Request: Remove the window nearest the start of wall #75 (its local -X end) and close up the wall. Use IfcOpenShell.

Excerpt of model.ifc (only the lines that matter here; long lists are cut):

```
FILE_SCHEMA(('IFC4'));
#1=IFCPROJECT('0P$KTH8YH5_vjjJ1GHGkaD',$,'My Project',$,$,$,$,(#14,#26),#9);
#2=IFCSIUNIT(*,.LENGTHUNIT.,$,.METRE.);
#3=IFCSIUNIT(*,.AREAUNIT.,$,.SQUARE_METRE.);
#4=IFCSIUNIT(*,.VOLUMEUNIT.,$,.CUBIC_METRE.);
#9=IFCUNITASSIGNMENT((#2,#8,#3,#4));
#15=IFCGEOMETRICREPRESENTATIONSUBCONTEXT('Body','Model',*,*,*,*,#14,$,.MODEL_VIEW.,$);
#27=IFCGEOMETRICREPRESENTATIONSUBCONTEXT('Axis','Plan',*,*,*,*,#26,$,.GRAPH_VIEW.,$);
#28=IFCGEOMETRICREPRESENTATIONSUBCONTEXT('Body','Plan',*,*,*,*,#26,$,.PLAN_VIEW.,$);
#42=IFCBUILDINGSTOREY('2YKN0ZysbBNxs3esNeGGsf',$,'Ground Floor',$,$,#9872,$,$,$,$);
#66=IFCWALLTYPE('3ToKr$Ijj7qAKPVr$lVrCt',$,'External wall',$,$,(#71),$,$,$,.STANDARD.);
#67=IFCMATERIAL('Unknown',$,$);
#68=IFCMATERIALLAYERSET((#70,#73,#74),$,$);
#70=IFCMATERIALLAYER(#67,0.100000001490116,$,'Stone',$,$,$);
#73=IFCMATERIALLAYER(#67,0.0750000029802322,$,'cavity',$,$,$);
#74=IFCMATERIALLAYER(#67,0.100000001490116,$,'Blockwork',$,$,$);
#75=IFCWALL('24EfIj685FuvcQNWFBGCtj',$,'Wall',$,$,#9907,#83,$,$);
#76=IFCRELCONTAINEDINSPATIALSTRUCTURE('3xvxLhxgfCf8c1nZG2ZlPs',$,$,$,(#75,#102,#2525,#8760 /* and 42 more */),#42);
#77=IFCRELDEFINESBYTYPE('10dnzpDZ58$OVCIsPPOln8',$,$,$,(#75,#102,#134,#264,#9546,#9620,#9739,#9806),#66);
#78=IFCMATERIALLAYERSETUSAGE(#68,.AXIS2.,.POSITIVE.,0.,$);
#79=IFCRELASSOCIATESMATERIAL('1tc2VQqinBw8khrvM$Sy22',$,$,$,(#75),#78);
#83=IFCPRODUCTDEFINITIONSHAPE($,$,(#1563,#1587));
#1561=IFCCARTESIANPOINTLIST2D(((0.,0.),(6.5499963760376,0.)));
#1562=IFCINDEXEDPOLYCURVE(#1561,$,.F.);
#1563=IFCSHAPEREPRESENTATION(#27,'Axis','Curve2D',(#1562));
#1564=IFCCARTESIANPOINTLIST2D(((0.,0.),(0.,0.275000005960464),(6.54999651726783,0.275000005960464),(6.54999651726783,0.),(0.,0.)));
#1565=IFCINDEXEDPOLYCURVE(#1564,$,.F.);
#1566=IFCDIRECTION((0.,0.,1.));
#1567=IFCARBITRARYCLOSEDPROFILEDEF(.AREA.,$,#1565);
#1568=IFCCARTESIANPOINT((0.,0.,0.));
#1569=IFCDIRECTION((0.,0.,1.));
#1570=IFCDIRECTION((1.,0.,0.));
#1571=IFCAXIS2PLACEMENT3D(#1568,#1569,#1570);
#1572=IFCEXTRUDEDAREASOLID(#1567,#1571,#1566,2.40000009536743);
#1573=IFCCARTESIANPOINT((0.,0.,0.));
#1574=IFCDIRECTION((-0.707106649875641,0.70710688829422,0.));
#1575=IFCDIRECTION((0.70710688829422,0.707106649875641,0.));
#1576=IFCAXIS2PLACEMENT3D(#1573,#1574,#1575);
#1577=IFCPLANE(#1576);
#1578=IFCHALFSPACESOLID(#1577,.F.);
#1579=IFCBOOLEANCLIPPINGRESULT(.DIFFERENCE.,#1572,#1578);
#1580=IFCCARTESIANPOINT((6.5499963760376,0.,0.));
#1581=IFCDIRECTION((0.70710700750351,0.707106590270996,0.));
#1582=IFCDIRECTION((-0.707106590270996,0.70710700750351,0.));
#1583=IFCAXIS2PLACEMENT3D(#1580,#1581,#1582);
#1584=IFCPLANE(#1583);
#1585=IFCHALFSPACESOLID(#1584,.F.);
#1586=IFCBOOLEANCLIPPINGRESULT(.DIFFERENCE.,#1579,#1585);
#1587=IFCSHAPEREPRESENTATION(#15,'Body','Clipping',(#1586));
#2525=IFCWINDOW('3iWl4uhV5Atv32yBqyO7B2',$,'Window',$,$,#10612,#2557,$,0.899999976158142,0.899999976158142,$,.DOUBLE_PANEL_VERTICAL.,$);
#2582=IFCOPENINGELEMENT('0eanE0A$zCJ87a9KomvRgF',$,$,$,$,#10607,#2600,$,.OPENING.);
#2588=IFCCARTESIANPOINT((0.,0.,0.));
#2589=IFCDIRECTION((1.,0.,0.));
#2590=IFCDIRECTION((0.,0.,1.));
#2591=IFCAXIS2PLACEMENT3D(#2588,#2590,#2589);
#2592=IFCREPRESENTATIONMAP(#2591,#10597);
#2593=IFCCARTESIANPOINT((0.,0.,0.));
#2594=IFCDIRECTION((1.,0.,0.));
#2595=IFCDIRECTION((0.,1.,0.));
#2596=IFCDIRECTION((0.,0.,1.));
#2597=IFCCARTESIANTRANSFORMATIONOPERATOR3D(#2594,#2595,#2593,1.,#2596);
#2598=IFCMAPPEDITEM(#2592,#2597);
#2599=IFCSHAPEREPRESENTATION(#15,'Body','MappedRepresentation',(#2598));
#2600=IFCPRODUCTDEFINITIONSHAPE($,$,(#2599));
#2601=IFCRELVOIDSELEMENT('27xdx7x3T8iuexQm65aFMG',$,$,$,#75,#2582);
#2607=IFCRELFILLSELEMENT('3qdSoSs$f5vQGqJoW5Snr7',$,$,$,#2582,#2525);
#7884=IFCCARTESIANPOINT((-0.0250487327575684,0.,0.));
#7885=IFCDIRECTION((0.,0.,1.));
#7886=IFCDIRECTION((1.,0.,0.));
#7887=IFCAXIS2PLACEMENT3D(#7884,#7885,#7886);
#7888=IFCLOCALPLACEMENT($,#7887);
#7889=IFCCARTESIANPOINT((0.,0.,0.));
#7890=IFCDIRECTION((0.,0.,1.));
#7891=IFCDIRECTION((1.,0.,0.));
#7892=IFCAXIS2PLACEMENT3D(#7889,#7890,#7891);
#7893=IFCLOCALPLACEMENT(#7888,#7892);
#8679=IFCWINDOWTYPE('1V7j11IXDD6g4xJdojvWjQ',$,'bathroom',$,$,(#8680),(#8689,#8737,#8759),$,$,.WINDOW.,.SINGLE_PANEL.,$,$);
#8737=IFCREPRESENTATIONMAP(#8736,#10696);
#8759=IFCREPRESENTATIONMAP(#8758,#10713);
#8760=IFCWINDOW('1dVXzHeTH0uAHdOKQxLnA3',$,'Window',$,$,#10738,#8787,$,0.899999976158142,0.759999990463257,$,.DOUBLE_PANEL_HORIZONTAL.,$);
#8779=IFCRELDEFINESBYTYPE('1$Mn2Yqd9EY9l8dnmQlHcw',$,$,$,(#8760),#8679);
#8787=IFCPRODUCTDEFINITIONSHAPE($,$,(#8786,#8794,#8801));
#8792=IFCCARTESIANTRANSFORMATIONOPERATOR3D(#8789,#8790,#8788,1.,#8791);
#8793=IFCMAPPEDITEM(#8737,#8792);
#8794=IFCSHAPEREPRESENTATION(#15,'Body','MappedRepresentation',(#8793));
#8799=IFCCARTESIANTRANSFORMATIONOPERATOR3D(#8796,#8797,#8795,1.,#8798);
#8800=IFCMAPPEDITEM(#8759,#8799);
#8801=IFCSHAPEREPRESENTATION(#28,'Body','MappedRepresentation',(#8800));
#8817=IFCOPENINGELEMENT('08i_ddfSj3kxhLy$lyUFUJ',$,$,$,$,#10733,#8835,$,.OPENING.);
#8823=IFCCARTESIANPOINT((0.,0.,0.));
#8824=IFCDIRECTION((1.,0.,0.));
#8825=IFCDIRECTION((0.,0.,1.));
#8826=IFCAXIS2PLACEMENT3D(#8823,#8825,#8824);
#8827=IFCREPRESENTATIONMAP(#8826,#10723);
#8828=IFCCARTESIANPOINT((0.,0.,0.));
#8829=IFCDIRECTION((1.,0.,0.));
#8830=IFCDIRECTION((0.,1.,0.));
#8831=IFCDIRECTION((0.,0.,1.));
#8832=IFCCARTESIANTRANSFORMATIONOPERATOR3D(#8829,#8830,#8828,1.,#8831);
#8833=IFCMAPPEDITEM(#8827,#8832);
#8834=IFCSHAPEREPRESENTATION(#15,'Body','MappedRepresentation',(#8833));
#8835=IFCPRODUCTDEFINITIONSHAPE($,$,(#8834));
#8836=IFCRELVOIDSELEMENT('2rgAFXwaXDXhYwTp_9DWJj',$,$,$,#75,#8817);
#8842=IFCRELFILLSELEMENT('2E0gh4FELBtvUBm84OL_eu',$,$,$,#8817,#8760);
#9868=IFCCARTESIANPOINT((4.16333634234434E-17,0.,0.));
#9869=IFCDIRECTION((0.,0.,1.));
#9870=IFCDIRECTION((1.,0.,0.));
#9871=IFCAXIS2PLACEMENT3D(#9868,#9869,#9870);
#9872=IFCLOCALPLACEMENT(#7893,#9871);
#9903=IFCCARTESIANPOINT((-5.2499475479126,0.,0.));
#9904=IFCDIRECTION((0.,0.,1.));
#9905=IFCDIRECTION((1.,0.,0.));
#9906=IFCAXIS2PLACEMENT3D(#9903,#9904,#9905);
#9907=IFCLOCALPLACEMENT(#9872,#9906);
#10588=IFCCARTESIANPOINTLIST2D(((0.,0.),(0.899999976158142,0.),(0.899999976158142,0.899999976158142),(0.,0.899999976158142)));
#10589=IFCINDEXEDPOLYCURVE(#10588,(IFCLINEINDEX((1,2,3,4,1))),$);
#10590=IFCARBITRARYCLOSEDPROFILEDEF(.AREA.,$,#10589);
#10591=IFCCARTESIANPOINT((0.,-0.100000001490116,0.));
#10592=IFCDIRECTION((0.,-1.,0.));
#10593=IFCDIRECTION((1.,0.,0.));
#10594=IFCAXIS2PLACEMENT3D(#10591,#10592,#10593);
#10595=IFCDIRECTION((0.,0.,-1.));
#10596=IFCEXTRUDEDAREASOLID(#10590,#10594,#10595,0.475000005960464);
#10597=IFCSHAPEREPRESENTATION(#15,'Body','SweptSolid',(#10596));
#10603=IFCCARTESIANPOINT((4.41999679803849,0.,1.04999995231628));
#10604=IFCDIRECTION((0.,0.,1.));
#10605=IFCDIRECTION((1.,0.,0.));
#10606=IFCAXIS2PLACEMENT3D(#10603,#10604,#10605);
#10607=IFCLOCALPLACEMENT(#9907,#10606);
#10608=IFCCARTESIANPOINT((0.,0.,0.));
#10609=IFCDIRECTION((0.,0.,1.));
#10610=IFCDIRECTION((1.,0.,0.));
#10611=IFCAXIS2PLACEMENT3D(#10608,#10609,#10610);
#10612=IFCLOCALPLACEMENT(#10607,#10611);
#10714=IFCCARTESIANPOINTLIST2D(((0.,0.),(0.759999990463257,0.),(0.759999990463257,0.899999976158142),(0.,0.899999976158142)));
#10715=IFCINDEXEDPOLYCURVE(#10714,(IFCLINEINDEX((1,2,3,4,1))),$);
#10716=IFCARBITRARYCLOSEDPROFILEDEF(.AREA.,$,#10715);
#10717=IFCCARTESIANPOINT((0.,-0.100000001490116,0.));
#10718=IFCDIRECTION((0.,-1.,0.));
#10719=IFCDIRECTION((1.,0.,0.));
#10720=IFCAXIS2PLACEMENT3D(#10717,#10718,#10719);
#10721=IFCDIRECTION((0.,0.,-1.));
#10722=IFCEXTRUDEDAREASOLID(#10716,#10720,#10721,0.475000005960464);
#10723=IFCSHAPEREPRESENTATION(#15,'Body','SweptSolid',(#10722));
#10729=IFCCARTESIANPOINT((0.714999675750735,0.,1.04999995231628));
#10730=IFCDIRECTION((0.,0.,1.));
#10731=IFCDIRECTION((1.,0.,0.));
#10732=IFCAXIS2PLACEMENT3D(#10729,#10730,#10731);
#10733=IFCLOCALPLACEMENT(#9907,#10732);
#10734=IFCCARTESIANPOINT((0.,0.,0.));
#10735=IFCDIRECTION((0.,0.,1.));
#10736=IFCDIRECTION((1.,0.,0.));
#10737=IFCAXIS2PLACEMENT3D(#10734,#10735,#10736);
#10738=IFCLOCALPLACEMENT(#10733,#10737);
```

```python
import ifcopenshell
import ifcopenshell.api.feature
import ifcopenshell.api.root
import ifcopenshell.geom
import ifcopenshell.util.shape

model = ifcopenshell.open("model.ifc")
settings = ifcopenshell.geom.settings()


def volume(element):
    """Net volume in cubic metres, openings subtracted."""
    shape = ifcopenshell.geom.create_shape(settings, element)
    return ifcopenshell.util.shape.get_volume(shape.geometry)


window = model.by_id(8760)
opening = window.FillsVoids[0].RelatingOpeningElement
wall = opening.VoidsElements[0].RelatingBuildingElement
before = volume(wall)

ifcopenshell.api.root.remove_product(model, product=window)
ifcopenshell.api.feature.remove_feature(model, feature=opening)

after = volume(wall)

print(f"wall volume {before:.3f} -> {after:.3f} m3")

model.write("model_rev.ifc")
```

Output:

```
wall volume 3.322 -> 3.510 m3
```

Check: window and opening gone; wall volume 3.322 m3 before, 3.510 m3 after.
